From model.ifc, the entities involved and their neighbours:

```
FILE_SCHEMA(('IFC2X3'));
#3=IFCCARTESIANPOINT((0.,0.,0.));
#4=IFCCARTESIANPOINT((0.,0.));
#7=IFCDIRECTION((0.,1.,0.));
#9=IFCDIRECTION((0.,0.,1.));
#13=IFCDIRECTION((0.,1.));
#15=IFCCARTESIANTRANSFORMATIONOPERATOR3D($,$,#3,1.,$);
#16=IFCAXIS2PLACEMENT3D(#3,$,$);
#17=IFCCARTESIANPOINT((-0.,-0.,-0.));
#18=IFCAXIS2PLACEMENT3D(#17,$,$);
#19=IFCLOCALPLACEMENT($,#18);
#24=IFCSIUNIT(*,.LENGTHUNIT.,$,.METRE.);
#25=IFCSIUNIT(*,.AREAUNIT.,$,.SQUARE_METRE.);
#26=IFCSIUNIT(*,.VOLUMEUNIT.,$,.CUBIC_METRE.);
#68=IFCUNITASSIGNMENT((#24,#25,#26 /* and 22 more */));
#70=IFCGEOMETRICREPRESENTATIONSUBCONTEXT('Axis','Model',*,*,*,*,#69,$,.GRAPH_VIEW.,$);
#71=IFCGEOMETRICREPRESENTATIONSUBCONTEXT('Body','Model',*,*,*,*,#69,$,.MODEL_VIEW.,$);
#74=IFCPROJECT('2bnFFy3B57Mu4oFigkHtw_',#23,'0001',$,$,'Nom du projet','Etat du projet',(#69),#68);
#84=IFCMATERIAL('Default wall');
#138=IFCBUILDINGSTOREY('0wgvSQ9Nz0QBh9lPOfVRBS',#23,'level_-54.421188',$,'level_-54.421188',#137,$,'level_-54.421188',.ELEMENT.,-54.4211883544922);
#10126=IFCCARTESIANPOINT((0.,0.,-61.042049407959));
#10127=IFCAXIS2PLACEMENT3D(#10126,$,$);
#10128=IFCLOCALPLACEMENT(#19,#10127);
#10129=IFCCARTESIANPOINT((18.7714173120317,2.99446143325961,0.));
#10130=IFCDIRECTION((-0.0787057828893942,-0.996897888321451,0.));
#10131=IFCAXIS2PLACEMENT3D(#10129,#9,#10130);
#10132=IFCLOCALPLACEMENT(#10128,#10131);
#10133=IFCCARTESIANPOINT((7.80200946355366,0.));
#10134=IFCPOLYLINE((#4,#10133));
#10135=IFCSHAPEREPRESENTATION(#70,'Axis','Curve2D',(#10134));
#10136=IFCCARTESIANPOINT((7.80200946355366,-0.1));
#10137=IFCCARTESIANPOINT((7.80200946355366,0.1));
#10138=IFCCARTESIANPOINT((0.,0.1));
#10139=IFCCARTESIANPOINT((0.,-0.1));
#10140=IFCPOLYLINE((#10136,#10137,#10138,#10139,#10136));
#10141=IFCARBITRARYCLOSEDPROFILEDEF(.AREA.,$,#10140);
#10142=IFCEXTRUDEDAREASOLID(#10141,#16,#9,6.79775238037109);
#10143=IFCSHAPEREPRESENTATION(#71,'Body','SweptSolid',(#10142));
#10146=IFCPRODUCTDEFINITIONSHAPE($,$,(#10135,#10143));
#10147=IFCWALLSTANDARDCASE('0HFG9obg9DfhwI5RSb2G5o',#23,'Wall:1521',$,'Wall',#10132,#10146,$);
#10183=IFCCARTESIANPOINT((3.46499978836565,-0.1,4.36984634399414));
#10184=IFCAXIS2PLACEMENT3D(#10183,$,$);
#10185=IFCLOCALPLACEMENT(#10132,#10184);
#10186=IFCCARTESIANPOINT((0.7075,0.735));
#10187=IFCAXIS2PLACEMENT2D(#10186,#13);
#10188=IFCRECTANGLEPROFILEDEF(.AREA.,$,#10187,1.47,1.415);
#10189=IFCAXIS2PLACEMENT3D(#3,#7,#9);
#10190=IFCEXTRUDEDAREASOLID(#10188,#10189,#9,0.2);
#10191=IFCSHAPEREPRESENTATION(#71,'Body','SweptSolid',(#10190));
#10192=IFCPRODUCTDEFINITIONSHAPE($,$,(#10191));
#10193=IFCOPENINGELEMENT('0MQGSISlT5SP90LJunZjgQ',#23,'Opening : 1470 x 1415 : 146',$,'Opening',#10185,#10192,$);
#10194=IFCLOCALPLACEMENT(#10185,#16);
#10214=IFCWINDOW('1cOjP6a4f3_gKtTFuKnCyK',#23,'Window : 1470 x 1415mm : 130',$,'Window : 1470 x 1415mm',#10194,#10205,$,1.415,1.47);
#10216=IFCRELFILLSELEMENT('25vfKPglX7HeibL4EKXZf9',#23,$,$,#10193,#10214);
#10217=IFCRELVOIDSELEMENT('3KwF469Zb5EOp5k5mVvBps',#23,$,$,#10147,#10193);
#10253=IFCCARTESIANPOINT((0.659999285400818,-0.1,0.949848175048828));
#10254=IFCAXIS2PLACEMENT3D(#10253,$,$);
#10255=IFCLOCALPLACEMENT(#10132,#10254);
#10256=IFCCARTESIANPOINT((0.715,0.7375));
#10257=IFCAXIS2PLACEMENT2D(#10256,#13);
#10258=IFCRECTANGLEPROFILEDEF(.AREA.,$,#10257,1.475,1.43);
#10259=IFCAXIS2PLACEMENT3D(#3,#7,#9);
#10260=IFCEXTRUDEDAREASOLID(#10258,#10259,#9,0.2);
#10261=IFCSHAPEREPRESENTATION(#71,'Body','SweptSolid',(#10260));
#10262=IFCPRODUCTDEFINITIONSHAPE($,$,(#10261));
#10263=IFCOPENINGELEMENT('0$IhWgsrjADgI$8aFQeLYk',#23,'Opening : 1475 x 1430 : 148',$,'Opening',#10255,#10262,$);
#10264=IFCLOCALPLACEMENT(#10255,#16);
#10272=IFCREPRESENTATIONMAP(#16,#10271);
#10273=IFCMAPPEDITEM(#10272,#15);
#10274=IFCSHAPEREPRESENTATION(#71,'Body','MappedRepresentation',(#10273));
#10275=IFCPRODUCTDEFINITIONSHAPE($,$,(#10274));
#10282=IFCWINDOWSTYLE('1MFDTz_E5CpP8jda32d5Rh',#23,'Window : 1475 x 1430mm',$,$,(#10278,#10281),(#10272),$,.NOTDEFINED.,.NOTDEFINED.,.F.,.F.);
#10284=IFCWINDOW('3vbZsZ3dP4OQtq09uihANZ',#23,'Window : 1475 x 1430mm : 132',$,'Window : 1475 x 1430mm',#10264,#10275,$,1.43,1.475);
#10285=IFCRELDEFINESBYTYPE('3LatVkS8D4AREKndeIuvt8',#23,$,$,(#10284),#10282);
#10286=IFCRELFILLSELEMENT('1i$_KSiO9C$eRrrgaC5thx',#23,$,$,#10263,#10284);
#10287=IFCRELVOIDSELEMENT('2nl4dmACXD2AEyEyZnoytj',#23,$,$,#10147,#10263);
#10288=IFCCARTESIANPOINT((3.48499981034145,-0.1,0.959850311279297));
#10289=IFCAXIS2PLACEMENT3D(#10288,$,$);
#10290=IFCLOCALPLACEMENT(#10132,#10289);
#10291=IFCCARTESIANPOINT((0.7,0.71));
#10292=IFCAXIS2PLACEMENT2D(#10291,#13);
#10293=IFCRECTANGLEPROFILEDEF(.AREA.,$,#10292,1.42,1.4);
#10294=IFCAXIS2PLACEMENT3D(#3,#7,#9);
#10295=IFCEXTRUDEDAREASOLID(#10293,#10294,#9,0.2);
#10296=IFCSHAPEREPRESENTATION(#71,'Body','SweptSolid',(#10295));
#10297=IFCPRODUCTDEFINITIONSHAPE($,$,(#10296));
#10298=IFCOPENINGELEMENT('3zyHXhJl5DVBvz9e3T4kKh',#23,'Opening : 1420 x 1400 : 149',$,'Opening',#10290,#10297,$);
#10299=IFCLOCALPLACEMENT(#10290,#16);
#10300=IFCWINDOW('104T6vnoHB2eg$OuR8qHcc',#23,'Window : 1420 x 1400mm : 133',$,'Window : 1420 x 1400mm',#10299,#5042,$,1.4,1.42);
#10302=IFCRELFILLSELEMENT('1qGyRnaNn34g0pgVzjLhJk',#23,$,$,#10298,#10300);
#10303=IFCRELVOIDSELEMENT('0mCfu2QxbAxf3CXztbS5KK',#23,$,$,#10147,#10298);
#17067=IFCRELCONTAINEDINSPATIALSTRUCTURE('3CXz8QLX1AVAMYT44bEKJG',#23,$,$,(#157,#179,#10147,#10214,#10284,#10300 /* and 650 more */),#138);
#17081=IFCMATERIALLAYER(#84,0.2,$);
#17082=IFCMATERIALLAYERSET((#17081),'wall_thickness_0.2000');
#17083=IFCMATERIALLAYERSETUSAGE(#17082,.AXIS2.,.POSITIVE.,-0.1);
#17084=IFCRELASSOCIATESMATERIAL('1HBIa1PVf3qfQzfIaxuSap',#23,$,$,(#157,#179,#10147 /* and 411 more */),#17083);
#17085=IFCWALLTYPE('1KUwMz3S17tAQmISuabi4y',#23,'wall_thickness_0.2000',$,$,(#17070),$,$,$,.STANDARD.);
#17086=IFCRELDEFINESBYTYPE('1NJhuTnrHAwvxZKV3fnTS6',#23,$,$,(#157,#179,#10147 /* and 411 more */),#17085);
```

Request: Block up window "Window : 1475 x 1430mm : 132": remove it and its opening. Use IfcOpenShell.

```python
import ifcopenshell
import ifcopenshell.api.feature
import ifcopenshell.api.root
import ifcopenshell.geom
import ifcopenshell.util.shape

model = ifcopenshell.open("model.ifc")
settings = ifcopenshell.geom.settings()


def volume(element):
    """Net volume in cubic metres, openings subtracted."""
    shape = ifcopenshell.geom.create_shape(settings, element)
    return ifcopenshell.util.shape.get_volume(shape.geometry)


window = model.by_id(10284)
opening = window.FillsVoids[0].RelatingOpeningElement
wall = opening.VoidsElements[0].RelatingBuildingElement
before = volume(wall)

ifcopenshell.api.root.remove_product(model, product=window)
ifcopenshell.api.feature.remove_feature(model, feature=opening)

after = volume(wall)

print(f"wall volume {before:.3f} -> {after:.3f} m3")

model.write("model_updated.ifc")
```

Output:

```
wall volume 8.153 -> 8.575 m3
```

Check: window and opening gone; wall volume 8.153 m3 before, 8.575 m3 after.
